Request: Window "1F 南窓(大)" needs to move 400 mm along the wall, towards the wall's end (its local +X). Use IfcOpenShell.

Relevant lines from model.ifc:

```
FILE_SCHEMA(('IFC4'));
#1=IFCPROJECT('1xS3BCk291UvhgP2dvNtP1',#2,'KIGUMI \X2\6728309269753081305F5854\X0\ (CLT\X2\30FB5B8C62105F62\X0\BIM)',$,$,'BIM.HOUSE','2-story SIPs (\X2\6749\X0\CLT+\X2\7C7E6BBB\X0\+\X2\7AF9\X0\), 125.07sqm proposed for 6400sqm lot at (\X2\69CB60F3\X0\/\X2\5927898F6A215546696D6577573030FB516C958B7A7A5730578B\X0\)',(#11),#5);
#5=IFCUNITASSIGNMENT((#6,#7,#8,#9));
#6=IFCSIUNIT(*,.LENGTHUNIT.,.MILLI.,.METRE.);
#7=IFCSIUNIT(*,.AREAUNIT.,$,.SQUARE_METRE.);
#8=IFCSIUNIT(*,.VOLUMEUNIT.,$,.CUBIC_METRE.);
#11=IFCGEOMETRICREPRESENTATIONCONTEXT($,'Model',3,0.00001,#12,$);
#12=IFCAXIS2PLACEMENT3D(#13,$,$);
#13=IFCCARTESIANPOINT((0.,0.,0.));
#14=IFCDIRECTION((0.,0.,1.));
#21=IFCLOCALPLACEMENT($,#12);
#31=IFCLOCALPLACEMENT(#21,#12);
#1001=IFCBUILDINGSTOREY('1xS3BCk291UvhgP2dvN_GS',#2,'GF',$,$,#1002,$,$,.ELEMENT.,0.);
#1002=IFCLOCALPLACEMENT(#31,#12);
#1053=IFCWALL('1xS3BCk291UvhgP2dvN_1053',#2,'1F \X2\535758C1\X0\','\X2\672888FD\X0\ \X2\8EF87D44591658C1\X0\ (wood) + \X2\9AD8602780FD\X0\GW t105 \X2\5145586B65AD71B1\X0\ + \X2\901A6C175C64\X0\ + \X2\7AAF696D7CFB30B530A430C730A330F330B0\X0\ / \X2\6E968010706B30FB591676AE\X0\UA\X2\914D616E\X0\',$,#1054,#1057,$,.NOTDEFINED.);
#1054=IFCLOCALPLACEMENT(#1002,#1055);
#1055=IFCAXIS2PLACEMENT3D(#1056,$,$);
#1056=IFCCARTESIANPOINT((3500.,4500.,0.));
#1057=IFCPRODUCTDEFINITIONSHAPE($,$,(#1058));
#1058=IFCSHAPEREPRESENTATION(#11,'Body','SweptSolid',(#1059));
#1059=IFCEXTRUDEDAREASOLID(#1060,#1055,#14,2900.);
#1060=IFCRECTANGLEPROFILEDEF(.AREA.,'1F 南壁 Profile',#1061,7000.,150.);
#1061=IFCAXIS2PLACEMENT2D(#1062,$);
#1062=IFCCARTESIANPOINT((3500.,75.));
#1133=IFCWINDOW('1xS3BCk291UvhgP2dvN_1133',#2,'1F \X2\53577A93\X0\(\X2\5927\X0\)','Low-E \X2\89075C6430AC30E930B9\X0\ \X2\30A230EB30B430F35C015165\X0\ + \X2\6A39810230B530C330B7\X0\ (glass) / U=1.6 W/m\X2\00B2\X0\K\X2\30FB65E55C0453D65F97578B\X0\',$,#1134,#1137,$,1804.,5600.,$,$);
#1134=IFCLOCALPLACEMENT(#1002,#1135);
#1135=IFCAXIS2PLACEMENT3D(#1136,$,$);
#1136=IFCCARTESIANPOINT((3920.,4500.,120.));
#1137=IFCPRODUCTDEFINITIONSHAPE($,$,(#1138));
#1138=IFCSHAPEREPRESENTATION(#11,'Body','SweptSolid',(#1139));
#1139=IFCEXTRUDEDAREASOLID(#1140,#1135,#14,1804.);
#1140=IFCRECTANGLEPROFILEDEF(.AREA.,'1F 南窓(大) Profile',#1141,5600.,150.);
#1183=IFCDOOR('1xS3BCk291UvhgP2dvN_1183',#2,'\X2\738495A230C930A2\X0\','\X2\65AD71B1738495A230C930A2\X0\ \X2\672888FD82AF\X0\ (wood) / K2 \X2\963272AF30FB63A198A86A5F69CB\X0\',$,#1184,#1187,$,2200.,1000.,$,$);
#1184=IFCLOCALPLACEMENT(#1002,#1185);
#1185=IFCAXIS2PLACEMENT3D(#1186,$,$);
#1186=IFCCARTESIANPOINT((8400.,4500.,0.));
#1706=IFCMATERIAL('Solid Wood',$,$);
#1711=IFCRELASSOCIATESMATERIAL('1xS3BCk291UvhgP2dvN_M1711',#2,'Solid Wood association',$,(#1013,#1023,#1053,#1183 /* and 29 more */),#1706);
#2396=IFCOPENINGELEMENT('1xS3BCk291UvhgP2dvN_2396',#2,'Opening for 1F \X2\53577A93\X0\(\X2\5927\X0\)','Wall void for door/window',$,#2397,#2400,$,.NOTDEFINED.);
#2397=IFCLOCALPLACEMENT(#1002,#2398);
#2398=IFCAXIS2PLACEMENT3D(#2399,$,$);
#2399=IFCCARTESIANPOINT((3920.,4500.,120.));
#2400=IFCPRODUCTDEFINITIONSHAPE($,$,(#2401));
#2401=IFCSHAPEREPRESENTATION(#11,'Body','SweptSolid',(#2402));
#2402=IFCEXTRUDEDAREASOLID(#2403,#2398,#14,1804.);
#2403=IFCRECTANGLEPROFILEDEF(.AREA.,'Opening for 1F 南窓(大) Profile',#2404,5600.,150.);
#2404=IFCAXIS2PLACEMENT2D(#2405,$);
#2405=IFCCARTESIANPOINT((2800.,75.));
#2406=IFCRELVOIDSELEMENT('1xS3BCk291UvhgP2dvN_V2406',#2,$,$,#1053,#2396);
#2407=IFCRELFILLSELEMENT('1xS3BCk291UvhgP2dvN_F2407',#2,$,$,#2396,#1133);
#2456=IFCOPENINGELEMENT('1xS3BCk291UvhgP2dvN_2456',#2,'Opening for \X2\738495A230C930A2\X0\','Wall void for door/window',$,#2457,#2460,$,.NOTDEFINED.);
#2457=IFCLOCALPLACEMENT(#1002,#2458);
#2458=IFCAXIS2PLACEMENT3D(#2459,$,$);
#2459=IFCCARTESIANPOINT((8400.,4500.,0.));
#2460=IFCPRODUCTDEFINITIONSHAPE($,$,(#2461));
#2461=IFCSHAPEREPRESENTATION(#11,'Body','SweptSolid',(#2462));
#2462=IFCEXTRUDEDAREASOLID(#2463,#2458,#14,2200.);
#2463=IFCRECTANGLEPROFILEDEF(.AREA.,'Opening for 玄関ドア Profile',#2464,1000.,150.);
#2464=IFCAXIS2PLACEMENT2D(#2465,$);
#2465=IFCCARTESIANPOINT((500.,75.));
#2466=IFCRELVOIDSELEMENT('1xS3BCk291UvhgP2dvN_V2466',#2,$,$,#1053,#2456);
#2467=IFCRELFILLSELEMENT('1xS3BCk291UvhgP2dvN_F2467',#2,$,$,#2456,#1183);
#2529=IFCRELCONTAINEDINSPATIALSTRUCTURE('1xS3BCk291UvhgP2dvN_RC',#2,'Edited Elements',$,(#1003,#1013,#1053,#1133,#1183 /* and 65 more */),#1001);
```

```python
import ifcopenshell
import ifcopenshell.api.geometry
import ifcopenshell.util.placement

model = ifcopenshell.open("model.ifc")

window = model.by_guid("1xS3BCk291UvhgP2dvN_1133")
opening = window.FillsVoids[0].RelatingOpeningElement
wall = opening.VoidsElements[0].RelatingBuildingElement

wall_matrix = ifcopenshell.util.placement.get_local_placement(wall.ObjectPlacement)
shift = wall_matrix[:3, 0] * 400.0
before = ifcopenshell.util.placement.get_local_placement(window.ObjectPlacement)[:3, 3].copy()

# The window is not placed relative to its opening, so move both.
for product in (opening, window):
    matrix = ifcopenshell.util.placement.get_local_placement(product.ObjectPlacement)
    matrix[:3, 3] += shift
    ifcopenshell.api.geometry.edit_object_placement(model, product=product, matrix=matrix, is_si=False)

after = ifcopenshell.util.placement.get_local_placement(window.ObjectPlacement)[:3, 3]
print("window moved by", (after - before).round(3) + 0.0)

model.write("model_updated.ifc")
```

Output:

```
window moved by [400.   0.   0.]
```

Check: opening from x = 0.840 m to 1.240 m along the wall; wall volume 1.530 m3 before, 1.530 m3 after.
